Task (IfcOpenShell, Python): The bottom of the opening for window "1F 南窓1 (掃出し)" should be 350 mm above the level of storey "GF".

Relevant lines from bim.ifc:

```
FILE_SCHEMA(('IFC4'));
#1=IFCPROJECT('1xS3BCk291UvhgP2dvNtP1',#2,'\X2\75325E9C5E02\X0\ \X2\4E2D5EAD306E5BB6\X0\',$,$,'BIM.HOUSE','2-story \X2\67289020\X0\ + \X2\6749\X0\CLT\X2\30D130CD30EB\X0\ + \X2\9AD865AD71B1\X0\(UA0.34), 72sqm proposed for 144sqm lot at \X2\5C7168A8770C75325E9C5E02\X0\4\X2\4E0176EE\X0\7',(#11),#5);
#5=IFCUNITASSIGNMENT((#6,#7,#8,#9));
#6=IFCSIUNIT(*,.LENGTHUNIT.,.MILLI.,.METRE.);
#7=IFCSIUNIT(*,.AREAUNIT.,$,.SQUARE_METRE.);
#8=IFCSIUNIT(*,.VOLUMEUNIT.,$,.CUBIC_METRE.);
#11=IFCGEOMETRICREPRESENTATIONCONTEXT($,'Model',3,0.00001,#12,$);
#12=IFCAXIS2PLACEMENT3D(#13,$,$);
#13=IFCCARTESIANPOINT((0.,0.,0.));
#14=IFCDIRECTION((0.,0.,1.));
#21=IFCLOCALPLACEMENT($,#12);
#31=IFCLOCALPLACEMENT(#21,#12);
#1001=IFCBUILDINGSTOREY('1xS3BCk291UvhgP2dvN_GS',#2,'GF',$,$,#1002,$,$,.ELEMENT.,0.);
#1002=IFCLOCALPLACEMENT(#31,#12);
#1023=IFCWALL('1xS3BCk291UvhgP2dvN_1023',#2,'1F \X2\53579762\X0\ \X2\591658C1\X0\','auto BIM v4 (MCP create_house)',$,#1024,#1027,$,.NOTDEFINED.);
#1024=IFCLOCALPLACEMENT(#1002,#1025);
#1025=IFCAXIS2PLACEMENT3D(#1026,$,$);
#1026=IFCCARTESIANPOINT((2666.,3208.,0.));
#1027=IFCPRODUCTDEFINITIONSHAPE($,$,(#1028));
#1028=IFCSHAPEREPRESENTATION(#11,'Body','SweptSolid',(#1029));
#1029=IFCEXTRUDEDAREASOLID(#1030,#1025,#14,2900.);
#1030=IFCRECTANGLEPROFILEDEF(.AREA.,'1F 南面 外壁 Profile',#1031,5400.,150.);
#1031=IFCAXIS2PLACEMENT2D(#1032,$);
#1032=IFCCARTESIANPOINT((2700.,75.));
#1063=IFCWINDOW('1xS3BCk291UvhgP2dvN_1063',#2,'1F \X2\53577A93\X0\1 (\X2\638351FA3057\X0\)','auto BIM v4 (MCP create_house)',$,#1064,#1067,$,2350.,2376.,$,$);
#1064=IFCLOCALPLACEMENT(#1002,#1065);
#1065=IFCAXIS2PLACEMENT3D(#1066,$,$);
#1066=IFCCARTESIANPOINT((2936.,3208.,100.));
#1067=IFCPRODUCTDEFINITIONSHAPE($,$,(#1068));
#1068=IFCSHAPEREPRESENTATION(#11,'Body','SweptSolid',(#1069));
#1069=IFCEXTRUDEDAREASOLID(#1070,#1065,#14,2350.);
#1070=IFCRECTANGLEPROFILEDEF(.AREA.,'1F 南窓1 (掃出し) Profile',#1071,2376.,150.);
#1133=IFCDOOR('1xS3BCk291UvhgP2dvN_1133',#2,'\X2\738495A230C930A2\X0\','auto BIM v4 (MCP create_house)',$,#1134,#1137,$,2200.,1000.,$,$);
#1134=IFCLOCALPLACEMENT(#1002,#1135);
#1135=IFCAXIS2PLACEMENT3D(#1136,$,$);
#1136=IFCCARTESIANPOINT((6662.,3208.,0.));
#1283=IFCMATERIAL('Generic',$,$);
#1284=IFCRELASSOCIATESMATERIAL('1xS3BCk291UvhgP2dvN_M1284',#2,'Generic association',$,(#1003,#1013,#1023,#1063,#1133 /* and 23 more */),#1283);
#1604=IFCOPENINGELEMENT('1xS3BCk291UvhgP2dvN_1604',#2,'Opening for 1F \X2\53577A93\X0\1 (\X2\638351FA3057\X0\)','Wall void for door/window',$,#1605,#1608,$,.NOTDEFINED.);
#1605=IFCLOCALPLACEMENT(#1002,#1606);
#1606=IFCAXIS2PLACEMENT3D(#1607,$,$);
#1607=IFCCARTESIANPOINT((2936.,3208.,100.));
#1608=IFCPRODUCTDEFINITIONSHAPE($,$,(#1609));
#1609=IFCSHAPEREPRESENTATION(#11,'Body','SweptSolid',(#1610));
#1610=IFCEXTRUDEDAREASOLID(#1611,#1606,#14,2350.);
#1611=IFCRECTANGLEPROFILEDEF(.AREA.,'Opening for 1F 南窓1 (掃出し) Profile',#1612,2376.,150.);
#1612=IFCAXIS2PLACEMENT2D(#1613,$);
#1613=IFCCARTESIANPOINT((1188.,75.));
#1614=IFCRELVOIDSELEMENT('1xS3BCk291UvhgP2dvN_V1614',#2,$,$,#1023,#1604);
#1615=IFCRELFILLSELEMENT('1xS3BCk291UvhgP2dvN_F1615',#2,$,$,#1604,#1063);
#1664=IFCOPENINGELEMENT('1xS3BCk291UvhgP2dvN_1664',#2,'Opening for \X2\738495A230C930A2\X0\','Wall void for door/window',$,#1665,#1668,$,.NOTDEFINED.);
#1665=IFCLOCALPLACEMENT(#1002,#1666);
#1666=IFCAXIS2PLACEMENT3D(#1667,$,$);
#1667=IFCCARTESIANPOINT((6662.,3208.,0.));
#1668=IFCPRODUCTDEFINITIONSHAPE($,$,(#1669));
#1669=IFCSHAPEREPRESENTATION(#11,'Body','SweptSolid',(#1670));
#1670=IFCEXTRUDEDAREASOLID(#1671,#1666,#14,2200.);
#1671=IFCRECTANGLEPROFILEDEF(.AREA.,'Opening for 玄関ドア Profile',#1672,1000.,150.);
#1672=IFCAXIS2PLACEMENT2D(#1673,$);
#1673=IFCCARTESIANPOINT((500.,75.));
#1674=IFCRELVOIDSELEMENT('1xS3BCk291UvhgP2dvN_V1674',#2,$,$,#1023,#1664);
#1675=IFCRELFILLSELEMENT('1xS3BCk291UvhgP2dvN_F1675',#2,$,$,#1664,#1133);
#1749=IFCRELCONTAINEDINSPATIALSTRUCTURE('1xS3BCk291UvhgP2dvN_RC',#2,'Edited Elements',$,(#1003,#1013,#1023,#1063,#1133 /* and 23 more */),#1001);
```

```python
import numpy as np
import ifcopenshell
import ifcopenshell.api.geometry
import ifcopenshell.geom
import ifcopenshell.util.element
import ifcopenshell.util.placement
import ifcopenshell.util.shape
import ifcopenshell.util.unit

model = ifcopenshell.open("bim.ifc")
unit_scale = ifcopenshell.util.unit.calculate_unit_scale(model)

window = model.by_id(1063)
opening = window.FillsVoids[0].RelatingOpeningElement
storey = ifcopenshell.util.element.get_container(window, ifc_class="IfcBuildingStorey")
level = ifcopenshell.util.placement.get_local_placement(storey.ObjectPlacement)[2, 3]

# The opening's origin need not be at the sill, so measure its lowest point.
shape = ifcopenshell.geom.create_shape(ifcopenshell.geom.settings(), opening)
bottom = ifcopenshell.util.shape.get_shape_bottom_elevation(shape, shape.geometry) / unit_scale
dz = level + 0.35 / unit_scale - bottom

shift = np.array([0.0, 0.0, dz])
# The window is not placed relative to its opening, so move both.
for product in (opening, window):
    matrix = ifcopenshell.util.placement.get_local_placement(product.ObjectPlacement)
    matrix[:3, 3] += shift
    ifcopenshell.api.geometry.edit_object_placement(model, product=product, matrix=matrix, is_si=False)

print(f"moved by {dz * unit_scale:+.3f} m")

model.write("bim_updated.ifc")
```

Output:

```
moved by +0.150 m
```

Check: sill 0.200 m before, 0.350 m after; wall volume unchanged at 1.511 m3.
